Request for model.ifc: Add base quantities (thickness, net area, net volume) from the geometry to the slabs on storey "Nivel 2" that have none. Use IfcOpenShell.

First a look at what the model holds.

```python
import ifcopenshell
import ifcopenshell.util.element
import ifcopenshell.util.unit

model = ifcopenshell.open("model.ifc")
print(model.schema)
for unit_type in ("LENGTHUNIT", "AREAUNIT", "VOLUMEUNIT"):
    print(unit_type, ifcopenshell.util.unit.calculate_unit_scale(model, unit_type))
storey = next(s for s in model.by_type("IfcBuildingStorey") if s.Name == "Nivel 2")
slabs = [e for e in ifcopenshell.util.element.get_decomposition(storey) if e.is_a("IfcSlab")]
for e in sorted(slabs, key=lambda e: e.id()):
    print(e.id(), e.is_a(), e.Name, list(ifcopenshell.util.element.get_psets(e, qtos_only=True)), sep=" | ")
```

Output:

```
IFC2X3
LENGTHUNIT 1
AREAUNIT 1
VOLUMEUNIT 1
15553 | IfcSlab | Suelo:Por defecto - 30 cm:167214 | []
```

```python
import ifcopenshell
import ifcopenshell.api.pset
import ifcopenshell.geom
import ifcopenshell.util.element
import ifcopenshell.util.shape
import ifcopenshell.util.unit

model = ifcopenshell.open("model.ifc")
unit_scale = ifcopenshell.util.unit.calculate_unit_scale(model)
area_scale = ifcopenshell.util.unit.calculate_unit_scale(model, "AREAUNIT")
volume_scale = ifcopenshell.util.unit.calculate_unit_scale(model, "VOLUMEUNIT")
settings = ifcopenshell.geom.settings()

storey = next(s for s in model.by_type("IfcBuildingStorey") if s.Name == "Nivel 2")
slabs = [e for e in ifcopenshell.util.element.get_decomposition(storey) if e.is_a("IfcSlab")]

for e in sorted(slabs, key=lambda e: e.id()):
    if ifcopenshell.util.element.get_psets(e, qtos_only=True, should_inherit=False):
        continue
    # Geometry comes back in metres, in the element's own axes.
    shape = ifcopenshell.geom.create_shape(settings, e)
    values = {
        "Width": ifcopenshell.util.shape.get_z(shape.geometry) / unit_scale,
        "NetArea": ifcopenshell.util.shape.get_footprint_area(shape.geometry) / area_scale,
        "NetVolume": ifcopenshell.util.shape.get_volume(shape.geometry) / volume_scale,
    }
    qto = ifcopenshell.api.pset.add_qto(model, product=e, name="BaseQuantities")
    ifcopenshell.api.pset.edit_qto(model, qto=qto, properties=values)
    print(e.id(), {k: round(v, 3) for k, v in values.items()})

model.write("model_edited.ifc")
```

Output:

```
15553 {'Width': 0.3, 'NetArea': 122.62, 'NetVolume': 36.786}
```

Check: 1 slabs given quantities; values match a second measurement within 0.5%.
